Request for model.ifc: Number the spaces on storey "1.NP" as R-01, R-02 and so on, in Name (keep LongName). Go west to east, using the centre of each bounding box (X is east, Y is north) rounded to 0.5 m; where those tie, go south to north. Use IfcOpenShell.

First a look at what the model holds.

```python
import ifcopenshell
import ifcopenshell.util.element
import ifcopenshell.util.placement

model = ifcopenshell.open("model.ifc")
print(model.schema)
storey = next(s for s in model.by_type("IfcBuildingStorey") if s.Name == "1.NP")
spaces = [e for e in ifcopenshell.util.element.get_decomposition(storey) if e.is_a("IfcSpace")]
for e in sorted(spaces, key=lambda e: e.id()):
    origin = ifcopenshell.util.placement.get_local_placement(e.ObjectPlacement)[:3, 3]
    print(e.id(), e.Name, e.LongName, origin.round(2) + 0.0, sep=" | ")
```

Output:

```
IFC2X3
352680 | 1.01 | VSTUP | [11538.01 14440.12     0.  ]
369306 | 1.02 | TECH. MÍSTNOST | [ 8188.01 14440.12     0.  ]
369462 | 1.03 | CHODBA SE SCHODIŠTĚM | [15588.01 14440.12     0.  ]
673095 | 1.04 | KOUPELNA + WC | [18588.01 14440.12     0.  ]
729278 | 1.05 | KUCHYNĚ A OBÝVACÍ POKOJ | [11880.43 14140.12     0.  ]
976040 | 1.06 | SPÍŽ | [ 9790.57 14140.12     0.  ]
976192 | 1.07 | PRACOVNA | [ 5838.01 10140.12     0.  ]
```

```python
import ifcopenshell
import ifcopenshell.geom
import ifcopenshell.util.element
import ifcopenshell.util.shape

model = ifcopenshell.open("model.ifc")
settings = ifcopenshell.geom.settings()
settings.set("use-world-coords", True)


def centre(element):
    shape = ifcopenshell.geom.create_shape(settings, element)
    return ifcopenshell.util.shape.get_bbox_centroid(shape.geometry)


storey = next(s for s in model.by_type("IfcBuildingStorey") if s.Name == "1.NP")
spaces = [e for e in ifcopenshell.util.element.get_decomposition(storey) if e.is_a("IfcSpace")]

# Insertion points can sit at a corner or the storey origin, so sort by the geometry (in metres).
centres = {e: centre(e) for e in spaces}
spaces.sort(key=lambda e: (round(centres[e][0] / 0.5), centres[e][1]))

for i, e in enumerate(spaces, start=1):
    number = f"R-{i:02d}"
    e.Name = number
    print(e.id(), number)

model.write("model_rev.ifc")
```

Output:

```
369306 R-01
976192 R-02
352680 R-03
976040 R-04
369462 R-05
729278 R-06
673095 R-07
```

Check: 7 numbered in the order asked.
